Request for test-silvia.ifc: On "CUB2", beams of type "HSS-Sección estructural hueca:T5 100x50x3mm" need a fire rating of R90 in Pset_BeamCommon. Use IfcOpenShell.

First a look at what the model holds.

```python
import ifcopenshell
import ifcopenshell.util.element

model = ifcopenshell.open("test-silvia.ifc")
print(model.schema)
storey = next(s for s in model.by_type("IfcBuildingStorey") if s.Name == "CUB2")
beams = [e for e in ifcopenshell.util.element.get_decomposition(storey) if e.is_a("IfcBeam")]
seen = {}
for e in beams:
    element_type = ifcopenshell.util.element.get_type(e)
    key = (element_type.Name if element_type != e and element_type else None, ifcopenshell.util.element.get_pset(e, "Pset_BeamCommon", "FireRating"))
    seen[key] = seen.get(key, 0) + 1
for (name, value), count in sorted(seen.items(), key=str):
    print(count, "x", name, "|", value)
```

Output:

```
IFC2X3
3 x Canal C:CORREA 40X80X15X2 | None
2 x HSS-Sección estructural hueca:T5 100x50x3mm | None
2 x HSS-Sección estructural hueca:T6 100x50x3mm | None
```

```python
import ifcopenshell
import ifcopenshell.api.pset
import ifcopenshell.util.element

model = ifcopenshell.open("test-silvia.ifc")

storey = next(s for s in model.by_type("IfcBuildingStorey") if s.Name == "CUB2")
beams = [e for e in ifcopenshell.util.element.get_decomposition(storey) if e.is_a("IfcBeam")]

count = 0
for e in beams:
    element_type = ifcopenshell.util.element.get_type(e)
    if element_type in (None, e) or element_type.Name != "HSS-Sección estructural hueca:T5 100x50x3mm":
        continue
    # add_pset returns the element's existing set when there is one.
    pset = ifcopenshell.api.pset.add_pset(model, product=e, name="Pset_BeamCommon")
    ifcopenshell.api.pset.edit_pset(model, pset=pset, properties={"FireRating": "R90"})
    count += 1

print(count, "beams updated")

model.write("test-silvia_updated.ifc")
```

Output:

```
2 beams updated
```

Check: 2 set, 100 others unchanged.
